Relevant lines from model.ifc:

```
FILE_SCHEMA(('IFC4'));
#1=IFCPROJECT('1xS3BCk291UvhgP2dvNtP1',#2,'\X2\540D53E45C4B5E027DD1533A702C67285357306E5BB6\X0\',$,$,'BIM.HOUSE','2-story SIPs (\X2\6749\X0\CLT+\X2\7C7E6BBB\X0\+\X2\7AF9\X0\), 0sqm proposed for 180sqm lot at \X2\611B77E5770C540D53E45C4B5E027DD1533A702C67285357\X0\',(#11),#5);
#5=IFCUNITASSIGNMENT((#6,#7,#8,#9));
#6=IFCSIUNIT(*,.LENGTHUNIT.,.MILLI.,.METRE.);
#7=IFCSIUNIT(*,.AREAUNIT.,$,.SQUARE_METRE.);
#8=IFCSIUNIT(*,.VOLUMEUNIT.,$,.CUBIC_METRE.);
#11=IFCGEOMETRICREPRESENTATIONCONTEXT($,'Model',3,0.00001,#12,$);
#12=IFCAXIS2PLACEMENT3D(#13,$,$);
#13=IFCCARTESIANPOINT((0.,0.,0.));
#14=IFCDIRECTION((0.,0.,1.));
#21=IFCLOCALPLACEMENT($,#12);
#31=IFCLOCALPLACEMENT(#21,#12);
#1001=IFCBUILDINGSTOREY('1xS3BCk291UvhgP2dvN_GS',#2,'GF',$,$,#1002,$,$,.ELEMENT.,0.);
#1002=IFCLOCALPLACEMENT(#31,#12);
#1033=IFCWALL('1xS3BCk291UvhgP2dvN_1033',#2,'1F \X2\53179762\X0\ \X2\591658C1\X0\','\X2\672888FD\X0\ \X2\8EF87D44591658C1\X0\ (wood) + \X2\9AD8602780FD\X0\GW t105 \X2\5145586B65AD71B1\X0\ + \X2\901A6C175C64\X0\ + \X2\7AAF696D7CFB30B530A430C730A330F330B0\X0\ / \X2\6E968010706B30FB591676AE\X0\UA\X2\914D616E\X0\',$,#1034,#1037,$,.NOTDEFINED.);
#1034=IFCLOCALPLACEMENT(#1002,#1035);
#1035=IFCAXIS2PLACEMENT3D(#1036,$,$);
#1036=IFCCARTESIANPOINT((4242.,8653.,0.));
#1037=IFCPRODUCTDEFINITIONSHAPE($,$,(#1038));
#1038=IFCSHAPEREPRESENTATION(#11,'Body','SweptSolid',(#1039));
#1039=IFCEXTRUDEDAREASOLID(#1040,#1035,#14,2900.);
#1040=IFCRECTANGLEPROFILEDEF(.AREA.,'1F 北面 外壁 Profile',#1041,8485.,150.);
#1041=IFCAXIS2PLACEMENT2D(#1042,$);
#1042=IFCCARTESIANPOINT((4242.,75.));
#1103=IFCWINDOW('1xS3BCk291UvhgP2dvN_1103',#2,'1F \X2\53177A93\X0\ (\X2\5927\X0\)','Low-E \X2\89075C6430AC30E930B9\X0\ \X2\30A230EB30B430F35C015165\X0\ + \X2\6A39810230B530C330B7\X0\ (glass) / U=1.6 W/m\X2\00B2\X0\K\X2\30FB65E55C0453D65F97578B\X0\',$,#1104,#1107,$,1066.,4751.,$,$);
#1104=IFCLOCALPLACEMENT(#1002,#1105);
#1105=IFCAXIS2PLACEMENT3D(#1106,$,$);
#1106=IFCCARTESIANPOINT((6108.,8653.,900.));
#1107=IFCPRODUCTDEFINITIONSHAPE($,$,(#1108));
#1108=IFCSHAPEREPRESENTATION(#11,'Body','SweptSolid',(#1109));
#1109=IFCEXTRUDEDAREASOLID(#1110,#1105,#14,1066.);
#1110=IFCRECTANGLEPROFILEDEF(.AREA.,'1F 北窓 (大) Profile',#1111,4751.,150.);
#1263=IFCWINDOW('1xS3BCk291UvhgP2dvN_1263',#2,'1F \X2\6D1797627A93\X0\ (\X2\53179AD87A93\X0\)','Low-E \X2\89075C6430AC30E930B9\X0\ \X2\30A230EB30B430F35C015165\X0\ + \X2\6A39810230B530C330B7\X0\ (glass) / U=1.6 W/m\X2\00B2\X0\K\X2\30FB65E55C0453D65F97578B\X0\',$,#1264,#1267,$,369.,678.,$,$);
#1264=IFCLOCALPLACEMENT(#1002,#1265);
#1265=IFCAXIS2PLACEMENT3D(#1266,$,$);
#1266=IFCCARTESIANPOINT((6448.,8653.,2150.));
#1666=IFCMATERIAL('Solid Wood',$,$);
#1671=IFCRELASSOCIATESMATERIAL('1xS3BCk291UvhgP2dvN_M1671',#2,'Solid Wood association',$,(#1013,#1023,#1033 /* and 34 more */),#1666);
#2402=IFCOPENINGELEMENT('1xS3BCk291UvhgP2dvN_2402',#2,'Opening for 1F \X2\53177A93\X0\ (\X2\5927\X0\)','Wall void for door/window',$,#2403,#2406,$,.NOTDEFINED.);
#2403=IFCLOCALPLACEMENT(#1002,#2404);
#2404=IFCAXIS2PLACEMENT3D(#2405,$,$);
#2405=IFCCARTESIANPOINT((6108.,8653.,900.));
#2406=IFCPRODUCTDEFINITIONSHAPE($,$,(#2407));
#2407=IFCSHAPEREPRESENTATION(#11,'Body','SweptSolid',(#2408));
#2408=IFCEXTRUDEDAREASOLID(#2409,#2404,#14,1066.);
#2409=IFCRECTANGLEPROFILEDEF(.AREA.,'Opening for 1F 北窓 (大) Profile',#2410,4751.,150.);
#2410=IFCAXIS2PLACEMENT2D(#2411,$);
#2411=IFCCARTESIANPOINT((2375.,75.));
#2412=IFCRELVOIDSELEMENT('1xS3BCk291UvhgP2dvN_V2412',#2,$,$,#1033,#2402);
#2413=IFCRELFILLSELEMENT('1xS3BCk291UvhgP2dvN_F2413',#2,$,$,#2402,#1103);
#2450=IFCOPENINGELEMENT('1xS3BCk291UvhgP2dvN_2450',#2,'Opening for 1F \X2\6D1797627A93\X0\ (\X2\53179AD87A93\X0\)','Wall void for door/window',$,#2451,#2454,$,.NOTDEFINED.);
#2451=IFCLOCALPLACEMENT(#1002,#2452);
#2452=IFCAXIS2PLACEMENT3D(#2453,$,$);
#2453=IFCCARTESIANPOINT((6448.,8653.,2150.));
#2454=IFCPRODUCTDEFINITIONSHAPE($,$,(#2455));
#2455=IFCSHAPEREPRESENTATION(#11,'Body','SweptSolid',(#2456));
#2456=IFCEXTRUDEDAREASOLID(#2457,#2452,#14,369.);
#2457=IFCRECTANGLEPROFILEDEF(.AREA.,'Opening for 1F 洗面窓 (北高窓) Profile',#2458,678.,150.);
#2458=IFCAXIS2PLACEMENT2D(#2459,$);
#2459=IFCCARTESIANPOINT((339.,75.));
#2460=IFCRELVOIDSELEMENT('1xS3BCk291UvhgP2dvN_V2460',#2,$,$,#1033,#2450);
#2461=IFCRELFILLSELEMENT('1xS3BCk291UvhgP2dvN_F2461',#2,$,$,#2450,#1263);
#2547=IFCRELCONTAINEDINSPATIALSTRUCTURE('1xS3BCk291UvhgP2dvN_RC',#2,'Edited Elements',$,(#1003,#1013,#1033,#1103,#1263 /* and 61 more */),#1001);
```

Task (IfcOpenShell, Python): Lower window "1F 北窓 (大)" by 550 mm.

```python
import numpy as np
import ifcopenshell
import ifcopenshell.api.geometry
import ifcopenshell.util.placement
import ifcopenshell.util.unit

model = ifcopenshell.open("model.ifc")
unit_scale = ifcopenshell.util.unit.calculate_unit_scale(model)

window = model.by_guid("1xS3BCk291UvhgP2dvN_1103")
opening = window.FillsVoids[0].RelatingOpeningElement
dz = -550.0

shift = np.array([0.0, 0.0, dz])
# The window is not placed relative to its opening, so move both.
for product in (opening, window):
    matrix = ifcopenshell.util.placement.get_local_placement(product.ObjectPlacement)
    matrix[:3, 3] += shift
    ifcopenshell.api.geometry.edit_object_placement(model, product=product, matrix=matrix, is_si=False)

print(f"moved by {dz * unit_scale:+.3f} m")

model.write("model_updated.ifc")
```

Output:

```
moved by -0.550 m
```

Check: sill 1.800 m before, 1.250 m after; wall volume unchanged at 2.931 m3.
